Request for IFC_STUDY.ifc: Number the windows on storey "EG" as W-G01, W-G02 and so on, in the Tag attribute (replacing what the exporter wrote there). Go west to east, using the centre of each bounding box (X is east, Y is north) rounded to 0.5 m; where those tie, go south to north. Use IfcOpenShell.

First a look at what the model holds.

```python
import ifcopenshell
import ifcopenshell.util.element
import ifcopenshell.util.placement

model = ifcopenshell.open("IFC_STUDY.ifc")
print(model.schema)
storey = next(s for s in model.by_type("IfcBuildingStorey") if s.Name == "EG")
windows = [e for e in ifcopenshell.util.element.get_decomposition(storey) if e.is_a("IfcWindow")]
for e in sorted(windows, key=lambda e: e.id()):
    origin = ifcopenshell.util.placement.get_local_placement(e.ObjectPlacement)[:3, 3]
    print(e.id(), e.Tag, e.Name, origin.round(2) + 0.0, sep=" | ")
```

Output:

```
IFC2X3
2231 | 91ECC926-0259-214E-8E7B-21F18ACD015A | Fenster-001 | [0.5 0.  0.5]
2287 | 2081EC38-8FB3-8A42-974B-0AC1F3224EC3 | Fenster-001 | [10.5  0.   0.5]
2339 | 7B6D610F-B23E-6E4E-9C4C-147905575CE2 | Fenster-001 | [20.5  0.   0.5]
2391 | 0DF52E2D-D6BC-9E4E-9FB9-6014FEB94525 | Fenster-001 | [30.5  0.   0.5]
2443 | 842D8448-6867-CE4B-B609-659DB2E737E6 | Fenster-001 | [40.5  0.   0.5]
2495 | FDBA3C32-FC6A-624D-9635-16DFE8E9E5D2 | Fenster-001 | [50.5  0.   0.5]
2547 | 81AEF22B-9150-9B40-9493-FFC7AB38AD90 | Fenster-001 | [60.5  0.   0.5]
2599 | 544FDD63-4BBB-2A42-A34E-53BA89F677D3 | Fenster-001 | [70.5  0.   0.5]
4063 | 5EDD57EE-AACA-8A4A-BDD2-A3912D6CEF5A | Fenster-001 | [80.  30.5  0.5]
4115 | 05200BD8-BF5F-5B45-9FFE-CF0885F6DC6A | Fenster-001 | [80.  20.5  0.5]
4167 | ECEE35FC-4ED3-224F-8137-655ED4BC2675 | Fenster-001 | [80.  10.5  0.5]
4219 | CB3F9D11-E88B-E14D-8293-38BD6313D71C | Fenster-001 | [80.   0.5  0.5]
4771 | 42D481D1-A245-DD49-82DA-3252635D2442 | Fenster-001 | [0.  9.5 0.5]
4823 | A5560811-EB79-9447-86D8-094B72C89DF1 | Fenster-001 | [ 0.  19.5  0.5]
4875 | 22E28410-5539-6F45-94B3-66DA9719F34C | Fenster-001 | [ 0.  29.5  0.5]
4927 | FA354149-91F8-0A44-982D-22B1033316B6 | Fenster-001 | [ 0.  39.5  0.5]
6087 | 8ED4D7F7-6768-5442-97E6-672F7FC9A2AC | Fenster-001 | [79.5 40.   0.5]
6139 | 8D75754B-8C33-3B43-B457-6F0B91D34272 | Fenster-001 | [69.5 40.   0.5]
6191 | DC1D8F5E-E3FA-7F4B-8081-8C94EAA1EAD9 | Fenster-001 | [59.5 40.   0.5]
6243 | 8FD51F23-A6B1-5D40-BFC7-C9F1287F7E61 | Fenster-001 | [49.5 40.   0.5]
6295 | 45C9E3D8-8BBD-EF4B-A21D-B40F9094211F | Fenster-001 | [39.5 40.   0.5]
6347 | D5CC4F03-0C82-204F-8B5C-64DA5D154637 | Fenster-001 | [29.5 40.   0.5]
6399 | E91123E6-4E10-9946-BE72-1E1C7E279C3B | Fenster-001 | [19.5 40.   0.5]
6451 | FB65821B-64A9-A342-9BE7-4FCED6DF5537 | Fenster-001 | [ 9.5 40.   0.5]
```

```python
import ifcopenshell
import ifcopenshell.geom
import ifcopenshell.util.element
import ifcopenshell.util.shape

model = ifcopenshell.open("IFC_STUDY.ifc")
settings = ifcopenshell.geom.settings()
settings.set("use-world-coords", True)


def centre(element):
    shape = ifcopenshell.geom.create_shape(settings, element)
    return ifcopenshell.util.shape.get_bbox_centroid(shape.geometry)


storey = next(s for s in model.by_type("IfcBuildingStorey") if s.Name == "EG")
windows = [e for e in ifcopenshell.util.element.get_decomposition(storey) if e.is_a("IfcWindow")]

# Insertion points can sit at a corner or the storey origin, so sort by the geometry (in metres).
centres = {e: centre(e) for e in windows}
windows.sort(key=lambda e: (round(centres[e][0] / 0.5), centres[e][1]))

for i, e in enumerate(windows, start=1):
    number = f"W-G{i:02d}"
    e.Tag = number
    print(e.id(), number)

model.write("IFC_STUDY_edited.ifc")
```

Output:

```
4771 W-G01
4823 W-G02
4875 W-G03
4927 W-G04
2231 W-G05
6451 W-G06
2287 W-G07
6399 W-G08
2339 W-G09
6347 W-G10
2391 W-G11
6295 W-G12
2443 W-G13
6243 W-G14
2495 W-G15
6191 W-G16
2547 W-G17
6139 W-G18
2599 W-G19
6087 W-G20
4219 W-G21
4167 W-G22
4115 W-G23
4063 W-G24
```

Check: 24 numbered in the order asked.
